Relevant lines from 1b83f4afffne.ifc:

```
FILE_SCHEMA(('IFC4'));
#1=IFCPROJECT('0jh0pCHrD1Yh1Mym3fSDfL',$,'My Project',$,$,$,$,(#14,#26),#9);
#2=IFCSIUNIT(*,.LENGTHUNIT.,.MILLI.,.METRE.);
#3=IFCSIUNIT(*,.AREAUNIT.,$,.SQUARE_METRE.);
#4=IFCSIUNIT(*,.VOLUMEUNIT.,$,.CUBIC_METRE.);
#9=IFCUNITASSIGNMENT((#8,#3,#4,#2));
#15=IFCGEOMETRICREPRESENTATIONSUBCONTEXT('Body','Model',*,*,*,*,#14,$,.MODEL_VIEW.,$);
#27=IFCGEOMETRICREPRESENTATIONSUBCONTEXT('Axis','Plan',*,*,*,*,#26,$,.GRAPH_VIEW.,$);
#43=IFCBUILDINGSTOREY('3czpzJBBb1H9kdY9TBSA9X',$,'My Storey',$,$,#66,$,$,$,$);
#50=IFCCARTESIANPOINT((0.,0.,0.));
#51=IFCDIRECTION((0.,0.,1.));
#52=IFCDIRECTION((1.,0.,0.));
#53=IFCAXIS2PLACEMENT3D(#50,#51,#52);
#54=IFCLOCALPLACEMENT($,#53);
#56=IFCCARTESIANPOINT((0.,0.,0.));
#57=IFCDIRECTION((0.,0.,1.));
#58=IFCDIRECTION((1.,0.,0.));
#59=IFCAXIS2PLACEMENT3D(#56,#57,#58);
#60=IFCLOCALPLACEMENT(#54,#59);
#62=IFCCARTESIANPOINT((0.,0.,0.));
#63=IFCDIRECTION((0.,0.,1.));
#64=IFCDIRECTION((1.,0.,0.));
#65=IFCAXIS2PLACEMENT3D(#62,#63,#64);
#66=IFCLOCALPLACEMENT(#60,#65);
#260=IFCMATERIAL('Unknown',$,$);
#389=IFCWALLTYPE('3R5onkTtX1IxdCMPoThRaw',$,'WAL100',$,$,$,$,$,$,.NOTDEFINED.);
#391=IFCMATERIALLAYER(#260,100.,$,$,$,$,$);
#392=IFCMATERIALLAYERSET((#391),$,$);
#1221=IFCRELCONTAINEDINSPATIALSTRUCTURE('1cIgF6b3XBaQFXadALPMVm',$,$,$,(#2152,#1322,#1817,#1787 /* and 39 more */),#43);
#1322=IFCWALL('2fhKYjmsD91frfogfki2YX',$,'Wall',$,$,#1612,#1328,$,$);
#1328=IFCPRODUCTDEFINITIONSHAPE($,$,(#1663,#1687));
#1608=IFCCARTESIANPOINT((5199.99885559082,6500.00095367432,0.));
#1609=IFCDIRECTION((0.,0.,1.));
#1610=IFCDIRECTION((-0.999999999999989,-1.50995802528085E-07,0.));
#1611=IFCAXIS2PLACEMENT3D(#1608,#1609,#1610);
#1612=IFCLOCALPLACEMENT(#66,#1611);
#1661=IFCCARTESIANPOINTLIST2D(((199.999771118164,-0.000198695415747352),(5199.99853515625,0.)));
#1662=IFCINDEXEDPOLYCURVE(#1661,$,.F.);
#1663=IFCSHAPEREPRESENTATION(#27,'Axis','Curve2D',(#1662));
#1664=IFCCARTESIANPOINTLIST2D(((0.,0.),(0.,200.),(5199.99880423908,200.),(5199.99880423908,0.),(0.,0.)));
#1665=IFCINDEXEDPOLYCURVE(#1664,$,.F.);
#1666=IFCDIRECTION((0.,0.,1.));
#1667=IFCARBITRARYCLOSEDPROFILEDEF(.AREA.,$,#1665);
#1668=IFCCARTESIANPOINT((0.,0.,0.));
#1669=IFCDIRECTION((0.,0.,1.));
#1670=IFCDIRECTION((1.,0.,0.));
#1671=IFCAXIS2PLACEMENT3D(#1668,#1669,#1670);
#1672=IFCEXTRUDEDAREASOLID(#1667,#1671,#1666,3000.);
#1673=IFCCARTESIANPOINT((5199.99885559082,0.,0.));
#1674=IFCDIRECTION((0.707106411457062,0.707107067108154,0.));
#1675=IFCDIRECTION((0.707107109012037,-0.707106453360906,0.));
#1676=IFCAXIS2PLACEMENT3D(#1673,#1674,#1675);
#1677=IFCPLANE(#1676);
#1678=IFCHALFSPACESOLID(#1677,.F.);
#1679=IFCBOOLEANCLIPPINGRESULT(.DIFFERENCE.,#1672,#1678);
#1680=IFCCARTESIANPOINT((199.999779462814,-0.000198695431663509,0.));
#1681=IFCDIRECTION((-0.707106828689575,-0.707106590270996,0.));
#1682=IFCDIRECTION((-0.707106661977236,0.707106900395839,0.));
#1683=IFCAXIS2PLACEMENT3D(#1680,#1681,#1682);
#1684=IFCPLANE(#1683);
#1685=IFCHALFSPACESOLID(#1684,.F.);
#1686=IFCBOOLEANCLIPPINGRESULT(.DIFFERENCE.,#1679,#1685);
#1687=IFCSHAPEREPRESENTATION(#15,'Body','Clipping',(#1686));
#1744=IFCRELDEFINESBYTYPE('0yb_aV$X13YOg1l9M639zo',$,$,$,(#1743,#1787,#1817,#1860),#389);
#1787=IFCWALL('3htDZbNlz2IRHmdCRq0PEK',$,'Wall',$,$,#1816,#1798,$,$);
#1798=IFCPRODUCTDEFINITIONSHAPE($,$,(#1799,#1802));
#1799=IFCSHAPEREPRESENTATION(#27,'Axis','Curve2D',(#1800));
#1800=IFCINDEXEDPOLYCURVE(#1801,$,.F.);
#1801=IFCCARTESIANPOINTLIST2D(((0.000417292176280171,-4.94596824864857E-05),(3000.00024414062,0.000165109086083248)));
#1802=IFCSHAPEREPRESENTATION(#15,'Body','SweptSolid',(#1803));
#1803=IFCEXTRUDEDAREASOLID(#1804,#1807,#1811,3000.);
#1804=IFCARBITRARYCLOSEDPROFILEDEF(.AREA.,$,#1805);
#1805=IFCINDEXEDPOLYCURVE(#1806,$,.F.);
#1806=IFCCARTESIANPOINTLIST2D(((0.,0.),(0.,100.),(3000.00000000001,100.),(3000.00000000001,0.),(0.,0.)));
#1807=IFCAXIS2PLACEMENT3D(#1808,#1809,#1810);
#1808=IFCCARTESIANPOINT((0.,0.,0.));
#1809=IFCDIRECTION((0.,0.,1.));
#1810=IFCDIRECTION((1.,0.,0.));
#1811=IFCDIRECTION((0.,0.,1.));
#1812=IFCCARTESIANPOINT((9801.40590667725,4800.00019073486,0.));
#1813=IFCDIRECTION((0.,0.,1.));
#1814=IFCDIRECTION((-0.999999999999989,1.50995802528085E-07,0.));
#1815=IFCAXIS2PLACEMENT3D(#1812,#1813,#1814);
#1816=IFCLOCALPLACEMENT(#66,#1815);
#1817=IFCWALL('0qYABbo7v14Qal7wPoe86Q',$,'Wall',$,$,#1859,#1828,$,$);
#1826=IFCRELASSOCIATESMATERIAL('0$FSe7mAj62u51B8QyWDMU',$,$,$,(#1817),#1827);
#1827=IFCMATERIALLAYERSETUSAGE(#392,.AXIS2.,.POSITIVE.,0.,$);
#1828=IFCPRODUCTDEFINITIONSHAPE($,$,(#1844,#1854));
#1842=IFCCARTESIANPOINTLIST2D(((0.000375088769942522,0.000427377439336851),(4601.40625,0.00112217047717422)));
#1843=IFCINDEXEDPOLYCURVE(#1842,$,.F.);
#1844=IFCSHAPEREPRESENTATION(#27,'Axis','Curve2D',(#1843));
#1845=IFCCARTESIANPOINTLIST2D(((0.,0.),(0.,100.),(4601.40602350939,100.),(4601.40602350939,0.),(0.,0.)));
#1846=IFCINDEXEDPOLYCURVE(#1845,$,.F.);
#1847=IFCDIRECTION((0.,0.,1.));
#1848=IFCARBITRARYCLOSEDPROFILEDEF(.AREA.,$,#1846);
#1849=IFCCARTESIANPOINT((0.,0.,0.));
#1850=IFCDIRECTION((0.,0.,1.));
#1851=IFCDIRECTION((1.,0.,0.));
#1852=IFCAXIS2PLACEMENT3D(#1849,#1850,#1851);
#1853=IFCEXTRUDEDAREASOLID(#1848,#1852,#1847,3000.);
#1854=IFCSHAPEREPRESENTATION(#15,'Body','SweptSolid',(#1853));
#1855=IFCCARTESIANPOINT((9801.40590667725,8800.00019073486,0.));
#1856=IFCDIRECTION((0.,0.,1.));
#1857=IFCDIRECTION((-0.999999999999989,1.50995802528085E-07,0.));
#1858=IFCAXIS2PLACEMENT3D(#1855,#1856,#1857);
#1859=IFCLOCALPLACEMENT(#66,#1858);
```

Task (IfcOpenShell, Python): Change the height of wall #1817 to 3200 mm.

```python
import ifcopenshell
import ifcopenshell.geom
import ifcopenshell.util.representation
import ifcopenshell.util.shape
import ifcopenshell.util.unit

model = ifcopenshell.open("1b83f4afffne.ifc")
unit_scale = ifcopenshell.util.unit.calculate_unit_scale(model)
settings = ifcopenshell.geom.settings()


def volume(element):
    """Net volume in cubic metres, openings subtracted."""
    shape = ifcopenshell.geom.create_shape(settings, element)
    return ifcopenshell.util.shape.get_volume(shape.geometry)


wall = model.by_id(1817)
before = volume(wall)

body = ifcopenshell.util.representation.get_representation(wall, "Model", "Body")
solid = body.Items[0]
old_height = solid.Depth
solid.Depth = 3.2 / unit_scale
after = volume(wall)

print(f"height {old_height:g} -> {solid.Depth:g}, volume {before:.3f} -> {after:.3f} m3")

model.write("1b83f4afffne-out.ifc")
```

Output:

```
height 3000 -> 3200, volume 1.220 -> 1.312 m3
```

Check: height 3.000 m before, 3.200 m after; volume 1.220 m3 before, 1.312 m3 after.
